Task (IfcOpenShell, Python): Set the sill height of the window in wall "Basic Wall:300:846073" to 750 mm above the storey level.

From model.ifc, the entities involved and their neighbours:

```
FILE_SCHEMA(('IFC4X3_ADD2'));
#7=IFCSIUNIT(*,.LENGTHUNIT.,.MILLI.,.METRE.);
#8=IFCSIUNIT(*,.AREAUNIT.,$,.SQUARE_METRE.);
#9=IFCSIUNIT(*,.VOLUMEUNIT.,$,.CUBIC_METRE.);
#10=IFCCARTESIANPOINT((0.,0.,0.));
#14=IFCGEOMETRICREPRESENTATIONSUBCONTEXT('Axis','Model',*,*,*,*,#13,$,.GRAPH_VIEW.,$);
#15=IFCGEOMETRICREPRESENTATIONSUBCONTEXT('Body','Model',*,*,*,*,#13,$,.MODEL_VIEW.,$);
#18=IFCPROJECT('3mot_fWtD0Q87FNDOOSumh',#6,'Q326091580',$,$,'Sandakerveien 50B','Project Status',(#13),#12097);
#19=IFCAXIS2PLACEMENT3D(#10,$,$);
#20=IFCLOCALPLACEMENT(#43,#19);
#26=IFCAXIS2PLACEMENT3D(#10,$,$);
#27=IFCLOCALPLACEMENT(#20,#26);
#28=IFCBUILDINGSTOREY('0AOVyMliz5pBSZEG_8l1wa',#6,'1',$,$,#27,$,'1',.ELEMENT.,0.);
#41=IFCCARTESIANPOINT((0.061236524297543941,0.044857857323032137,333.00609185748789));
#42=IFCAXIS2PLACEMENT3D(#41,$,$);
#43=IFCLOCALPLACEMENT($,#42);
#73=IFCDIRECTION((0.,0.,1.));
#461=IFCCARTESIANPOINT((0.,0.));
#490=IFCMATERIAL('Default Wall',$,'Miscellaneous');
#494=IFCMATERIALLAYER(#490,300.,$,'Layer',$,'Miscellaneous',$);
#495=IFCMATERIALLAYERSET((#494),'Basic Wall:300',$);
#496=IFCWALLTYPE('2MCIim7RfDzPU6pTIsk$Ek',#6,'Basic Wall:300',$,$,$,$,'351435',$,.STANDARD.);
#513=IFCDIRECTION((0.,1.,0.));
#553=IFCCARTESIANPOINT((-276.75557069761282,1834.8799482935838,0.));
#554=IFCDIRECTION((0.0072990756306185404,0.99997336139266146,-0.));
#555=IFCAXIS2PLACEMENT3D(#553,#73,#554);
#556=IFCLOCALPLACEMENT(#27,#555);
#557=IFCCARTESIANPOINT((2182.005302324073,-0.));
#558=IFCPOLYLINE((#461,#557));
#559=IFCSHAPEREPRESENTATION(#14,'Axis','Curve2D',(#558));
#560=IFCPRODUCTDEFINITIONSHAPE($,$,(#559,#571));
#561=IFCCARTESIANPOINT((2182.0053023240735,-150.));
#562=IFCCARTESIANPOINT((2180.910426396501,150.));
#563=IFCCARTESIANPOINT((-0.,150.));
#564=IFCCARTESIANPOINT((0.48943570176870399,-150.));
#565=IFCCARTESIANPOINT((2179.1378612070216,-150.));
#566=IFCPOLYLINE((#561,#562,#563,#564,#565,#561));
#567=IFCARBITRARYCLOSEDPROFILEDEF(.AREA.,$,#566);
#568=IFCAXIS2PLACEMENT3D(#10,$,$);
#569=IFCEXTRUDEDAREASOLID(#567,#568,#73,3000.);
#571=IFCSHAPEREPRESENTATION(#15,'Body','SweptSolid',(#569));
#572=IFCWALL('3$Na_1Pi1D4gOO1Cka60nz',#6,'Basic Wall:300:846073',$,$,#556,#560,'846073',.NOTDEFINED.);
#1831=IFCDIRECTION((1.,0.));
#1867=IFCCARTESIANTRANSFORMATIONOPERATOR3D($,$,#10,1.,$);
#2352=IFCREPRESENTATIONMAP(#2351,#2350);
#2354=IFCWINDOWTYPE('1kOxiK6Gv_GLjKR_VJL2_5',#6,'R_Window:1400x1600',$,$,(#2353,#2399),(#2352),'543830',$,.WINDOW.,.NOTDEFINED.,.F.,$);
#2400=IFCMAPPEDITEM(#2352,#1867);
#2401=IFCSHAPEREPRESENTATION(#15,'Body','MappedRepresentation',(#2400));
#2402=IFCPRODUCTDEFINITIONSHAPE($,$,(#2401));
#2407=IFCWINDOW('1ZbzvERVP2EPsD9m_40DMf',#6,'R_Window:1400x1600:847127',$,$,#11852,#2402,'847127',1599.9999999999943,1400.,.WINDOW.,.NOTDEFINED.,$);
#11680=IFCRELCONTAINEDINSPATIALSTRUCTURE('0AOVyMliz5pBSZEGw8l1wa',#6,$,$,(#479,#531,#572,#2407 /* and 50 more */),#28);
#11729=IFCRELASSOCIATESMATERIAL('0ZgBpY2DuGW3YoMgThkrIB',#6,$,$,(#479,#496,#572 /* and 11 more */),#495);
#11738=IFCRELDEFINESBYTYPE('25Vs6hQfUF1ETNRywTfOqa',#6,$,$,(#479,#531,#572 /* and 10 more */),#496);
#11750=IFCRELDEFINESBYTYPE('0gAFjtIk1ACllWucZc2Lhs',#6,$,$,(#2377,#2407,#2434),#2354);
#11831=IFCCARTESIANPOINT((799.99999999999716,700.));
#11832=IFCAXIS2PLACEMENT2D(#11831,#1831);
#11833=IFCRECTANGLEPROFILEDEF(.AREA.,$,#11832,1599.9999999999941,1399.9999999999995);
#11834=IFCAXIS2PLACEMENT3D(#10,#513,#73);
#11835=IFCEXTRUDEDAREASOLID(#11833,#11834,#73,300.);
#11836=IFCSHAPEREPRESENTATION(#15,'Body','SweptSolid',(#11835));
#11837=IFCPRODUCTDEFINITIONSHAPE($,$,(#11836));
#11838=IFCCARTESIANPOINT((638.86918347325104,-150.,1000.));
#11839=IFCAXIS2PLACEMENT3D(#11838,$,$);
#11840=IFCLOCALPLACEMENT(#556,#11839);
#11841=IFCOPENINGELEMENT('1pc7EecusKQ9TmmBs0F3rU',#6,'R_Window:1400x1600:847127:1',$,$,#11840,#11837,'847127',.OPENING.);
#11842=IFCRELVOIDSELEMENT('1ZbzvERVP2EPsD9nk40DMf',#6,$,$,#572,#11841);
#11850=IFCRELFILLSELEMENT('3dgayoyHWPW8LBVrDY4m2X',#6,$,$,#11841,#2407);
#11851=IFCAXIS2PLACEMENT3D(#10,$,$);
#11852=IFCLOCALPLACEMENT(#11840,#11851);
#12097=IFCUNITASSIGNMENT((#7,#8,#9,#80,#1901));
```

```python
import numpy as np
import ifcopenshell
import ifcopenshell.api.geometry
import ifcopenshell.geom
import ifcopenshell.util.element
import ifcopenshell.util.placement
import ifcopenshell.util.shape
import ifcopenshell.util.unit

model = ifcopenshell.open("model.ifc")
unit_scale = ifcopenshell.util.unit.calculate_unit_scale(model)

window = model.by_guid("1ZbzvERVP2EPsD9m_40DMf")
opening = window.FillsVoids[0].RelatingOpeningElement
storey = ifcopenshell.util.element.get_container(window, ifc_class="IfcBuildingStorey")
level = ifcopenshell.util.placement.get_local_placement(storey.ObjectPlacement)[2, 3]

# The opening's origin need not be at the sill, so measure its lowest point.
shape = ifcopenshell.geom.create_shape(ifcopenshell.geom.settings(), opening)
bottom = ifcopenshell.util.shape.get_shape_bottom_elevation(shape, shape.geometry) / unit_scale
dz = level + 0.75 / unit_scale - bottom

shift = np.array([0.0, 0.0, dz])
# The window is placed relative to its opening, so it follows when the opening moves.
matrix = ifcopenshell.util.placement.get_local_placement(opening.ObjectPlacement)
matrix[:3, 3] += shift
ifcopenshell.api.geometry.edit_object_placement(
    model, product=opening, matrix=matrix, is_si=False, should_transform_children=True
)

print(f"moved by {dz * unit_scale:+.3f} m")

model.write("model-out.ifc")
```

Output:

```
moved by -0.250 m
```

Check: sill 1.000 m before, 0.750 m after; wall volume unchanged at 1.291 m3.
